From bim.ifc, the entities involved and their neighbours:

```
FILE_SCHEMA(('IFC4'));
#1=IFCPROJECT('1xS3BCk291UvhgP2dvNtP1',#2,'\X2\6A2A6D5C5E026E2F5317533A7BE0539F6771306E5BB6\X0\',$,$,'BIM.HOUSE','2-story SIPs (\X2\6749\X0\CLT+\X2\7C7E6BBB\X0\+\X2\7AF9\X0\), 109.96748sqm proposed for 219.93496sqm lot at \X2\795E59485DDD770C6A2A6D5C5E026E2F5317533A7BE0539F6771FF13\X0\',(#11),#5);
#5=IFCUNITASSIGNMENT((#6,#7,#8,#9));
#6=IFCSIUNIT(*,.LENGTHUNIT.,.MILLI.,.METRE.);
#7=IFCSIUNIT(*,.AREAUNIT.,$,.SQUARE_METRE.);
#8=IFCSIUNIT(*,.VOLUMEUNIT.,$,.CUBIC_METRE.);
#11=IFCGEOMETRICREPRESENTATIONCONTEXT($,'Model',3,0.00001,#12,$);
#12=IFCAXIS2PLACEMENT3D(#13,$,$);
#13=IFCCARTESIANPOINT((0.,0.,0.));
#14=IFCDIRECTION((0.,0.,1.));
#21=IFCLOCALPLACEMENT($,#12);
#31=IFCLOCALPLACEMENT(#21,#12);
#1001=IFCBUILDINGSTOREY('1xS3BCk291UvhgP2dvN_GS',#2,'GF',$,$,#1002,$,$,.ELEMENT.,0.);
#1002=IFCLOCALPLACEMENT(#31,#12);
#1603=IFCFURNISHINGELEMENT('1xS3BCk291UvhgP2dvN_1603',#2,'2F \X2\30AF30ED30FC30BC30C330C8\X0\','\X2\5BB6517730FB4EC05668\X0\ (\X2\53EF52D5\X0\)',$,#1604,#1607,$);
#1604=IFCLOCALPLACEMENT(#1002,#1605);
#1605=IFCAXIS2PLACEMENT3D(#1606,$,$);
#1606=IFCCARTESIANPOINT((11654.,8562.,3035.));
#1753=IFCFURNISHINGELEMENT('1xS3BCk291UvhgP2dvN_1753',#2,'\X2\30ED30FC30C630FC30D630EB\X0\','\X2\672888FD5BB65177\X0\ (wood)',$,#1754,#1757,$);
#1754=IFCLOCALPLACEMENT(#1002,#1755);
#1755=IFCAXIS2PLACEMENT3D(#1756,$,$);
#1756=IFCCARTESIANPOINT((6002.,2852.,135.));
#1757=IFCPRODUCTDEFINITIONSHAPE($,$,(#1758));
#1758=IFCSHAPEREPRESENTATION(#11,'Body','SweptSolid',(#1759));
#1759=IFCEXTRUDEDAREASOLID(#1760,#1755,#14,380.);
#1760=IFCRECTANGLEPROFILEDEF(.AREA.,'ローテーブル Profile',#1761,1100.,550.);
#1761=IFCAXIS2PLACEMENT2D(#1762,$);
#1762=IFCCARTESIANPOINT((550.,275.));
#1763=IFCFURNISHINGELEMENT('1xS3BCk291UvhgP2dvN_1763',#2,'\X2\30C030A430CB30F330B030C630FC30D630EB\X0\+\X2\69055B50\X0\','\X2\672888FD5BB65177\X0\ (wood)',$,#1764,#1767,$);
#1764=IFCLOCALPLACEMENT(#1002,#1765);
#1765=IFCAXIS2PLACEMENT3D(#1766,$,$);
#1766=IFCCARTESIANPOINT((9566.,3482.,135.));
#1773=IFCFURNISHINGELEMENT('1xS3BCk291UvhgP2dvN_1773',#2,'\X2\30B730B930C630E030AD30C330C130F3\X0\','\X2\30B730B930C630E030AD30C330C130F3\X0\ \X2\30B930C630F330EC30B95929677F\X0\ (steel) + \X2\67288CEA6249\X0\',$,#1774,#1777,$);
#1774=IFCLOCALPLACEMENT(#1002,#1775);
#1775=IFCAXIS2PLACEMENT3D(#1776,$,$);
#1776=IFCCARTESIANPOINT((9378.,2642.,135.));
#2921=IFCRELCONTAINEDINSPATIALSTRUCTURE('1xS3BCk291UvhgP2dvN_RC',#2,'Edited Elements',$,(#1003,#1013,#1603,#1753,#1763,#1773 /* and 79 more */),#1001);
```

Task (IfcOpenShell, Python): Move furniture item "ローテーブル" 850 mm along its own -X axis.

```python
import ifcopenshell
import ifcopenshell.api.geometry
import ifcopenshell.util.placement

model = ifcopenshell.open("bim.ifc")

item = model.by_guid("1xS3BCk291UvhgP2dvN_1753")
matrix = ifcopenshell.util.placement.get_local_placement(item.ObjectPlacement)
matrix[:3, 3] -= matrix[:3, 0] * 850.0
ifcopenshell.api.geometry.edit_object_placement(model, product=item, matrix=matrix, is_si=False)

print(ifcopenshell.util.placement.get_local_placement(item.ObjectPlacement).round(3) + 0.0)

model.write("bim-out.ifc")
```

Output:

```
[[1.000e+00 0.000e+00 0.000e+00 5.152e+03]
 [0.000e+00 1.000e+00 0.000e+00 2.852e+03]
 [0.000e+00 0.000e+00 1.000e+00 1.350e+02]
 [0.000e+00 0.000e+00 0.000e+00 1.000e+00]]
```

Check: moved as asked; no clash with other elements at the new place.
